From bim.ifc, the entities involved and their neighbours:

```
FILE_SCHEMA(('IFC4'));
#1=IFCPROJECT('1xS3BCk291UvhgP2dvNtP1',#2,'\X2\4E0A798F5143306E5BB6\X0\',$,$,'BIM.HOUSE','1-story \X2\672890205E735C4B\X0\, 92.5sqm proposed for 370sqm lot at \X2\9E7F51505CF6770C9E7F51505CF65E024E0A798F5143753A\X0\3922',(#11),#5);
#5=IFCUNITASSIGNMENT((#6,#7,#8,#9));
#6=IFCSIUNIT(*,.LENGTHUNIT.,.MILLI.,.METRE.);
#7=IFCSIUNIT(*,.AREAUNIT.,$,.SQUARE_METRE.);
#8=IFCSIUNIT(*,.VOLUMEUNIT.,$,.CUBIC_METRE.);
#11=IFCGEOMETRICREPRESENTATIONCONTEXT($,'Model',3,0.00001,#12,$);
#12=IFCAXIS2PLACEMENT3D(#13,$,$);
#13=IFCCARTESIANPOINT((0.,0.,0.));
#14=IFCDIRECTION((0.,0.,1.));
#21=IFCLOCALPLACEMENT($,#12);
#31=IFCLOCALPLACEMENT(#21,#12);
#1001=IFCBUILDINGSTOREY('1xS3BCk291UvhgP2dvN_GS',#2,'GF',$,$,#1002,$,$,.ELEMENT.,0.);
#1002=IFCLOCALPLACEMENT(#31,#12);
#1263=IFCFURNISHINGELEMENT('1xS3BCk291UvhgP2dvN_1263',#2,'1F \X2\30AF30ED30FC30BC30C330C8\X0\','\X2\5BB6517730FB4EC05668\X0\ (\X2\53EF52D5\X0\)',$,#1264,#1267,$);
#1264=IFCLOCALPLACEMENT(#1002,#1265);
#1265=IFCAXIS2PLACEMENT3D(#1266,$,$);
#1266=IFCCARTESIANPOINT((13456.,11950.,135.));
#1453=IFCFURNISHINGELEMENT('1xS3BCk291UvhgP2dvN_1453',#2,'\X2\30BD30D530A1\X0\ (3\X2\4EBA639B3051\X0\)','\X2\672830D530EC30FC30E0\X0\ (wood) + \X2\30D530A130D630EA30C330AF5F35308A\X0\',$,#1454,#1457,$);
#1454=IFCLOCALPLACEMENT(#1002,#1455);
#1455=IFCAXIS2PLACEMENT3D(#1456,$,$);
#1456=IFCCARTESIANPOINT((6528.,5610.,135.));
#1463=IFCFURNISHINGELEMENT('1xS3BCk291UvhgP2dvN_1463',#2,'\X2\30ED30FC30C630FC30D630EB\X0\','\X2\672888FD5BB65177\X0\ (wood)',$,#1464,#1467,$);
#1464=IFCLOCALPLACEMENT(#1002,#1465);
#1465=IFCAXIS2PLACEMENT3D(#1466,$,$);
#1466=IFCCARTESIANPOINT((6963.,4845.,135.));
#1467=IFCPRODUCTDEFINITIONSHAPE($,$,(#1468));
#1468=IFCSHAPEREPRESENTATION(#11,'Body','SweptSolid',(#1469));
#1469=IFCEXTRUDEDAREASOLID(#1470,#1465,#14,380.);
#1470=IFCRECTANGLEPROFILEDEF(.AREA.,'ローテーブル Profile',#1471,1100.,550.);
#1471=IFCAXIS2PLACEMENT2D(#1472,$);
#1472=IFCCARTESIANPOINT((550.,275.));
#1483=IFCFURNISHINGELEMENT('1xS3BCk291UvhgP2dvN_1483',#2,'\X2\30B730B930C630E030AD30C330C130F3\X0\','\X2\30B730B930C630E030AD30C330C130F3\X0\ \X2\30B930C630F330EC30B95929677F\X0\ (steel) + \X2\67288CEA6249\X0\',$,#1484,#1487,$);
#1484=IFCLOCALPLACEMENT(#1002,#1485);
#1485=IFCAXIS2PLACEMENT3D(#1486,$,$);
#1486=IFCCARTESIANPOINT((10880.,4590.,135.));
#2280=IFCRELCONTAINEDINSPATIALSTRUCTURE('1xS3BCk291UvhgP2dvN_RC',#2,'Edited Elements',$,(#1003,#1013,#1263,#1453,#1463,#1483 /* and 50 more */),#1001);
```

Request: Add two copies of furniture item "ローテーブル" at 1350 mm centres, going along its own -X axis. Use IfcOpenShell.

```python
import ifcopenshell
import ifcopenshell.api.geometry
import ifcopenshell.api.root
import ifcopenshell.util.element
import ifcopenshell.util.placement
import ifcopenshell.util.unit

model = ifcopenshell.open("bim.ifc")
unit_scale = ifcopenshell.util.unit.calculate_unit_scale(model)


def reuse_history(source, copy):
    """copy_class also copies each property set's owner history, people and application; keep the originals."""
    for rel in copy.IsDefinedBy:
        if rel.is_a("IfcRelDefinesByProperties") and (history := rel.RelatingPropertyDefinition.OwnerHistory):
            rel.RelatingPropertyDefinition.OwnerHistory = source.OwnerHistory
            ifcopenshell.util.element.remove_deep2(model, history)


source = model.by_guid("1xS3BCk291UvhgP2dvN_1463")
base = ifcopenshell.util.placement.get_local_placement(source.ObjectPlacement)
step = -base[:3, 0] * 1.35 / unit_scale

for i in range(1, 3):
    copy = ifcopenshell.api.root.copy_class(model, product=source)
    copy.Representation = ifcopenshell.util.element.copy_deep(
        model, source.Representation, exclude=["IfcGeometricRepresentationContext", "IfcRepresentationMap"]
    )
    reuse_history(source, copy)
    matrix = base.copy()
    matrix[:3, 3] += i * step
    print("added at", matrix[:3, 3].round(3) + 0.0)
    ifcopenshell.api.geometry.edit_object_placement(model, product=copy, matrix=matrix, is_si=False)

model.write("bim_rev.ifc")
```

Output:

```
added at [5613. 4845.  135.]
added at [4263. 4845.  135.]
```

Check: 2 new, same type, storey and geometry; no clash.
